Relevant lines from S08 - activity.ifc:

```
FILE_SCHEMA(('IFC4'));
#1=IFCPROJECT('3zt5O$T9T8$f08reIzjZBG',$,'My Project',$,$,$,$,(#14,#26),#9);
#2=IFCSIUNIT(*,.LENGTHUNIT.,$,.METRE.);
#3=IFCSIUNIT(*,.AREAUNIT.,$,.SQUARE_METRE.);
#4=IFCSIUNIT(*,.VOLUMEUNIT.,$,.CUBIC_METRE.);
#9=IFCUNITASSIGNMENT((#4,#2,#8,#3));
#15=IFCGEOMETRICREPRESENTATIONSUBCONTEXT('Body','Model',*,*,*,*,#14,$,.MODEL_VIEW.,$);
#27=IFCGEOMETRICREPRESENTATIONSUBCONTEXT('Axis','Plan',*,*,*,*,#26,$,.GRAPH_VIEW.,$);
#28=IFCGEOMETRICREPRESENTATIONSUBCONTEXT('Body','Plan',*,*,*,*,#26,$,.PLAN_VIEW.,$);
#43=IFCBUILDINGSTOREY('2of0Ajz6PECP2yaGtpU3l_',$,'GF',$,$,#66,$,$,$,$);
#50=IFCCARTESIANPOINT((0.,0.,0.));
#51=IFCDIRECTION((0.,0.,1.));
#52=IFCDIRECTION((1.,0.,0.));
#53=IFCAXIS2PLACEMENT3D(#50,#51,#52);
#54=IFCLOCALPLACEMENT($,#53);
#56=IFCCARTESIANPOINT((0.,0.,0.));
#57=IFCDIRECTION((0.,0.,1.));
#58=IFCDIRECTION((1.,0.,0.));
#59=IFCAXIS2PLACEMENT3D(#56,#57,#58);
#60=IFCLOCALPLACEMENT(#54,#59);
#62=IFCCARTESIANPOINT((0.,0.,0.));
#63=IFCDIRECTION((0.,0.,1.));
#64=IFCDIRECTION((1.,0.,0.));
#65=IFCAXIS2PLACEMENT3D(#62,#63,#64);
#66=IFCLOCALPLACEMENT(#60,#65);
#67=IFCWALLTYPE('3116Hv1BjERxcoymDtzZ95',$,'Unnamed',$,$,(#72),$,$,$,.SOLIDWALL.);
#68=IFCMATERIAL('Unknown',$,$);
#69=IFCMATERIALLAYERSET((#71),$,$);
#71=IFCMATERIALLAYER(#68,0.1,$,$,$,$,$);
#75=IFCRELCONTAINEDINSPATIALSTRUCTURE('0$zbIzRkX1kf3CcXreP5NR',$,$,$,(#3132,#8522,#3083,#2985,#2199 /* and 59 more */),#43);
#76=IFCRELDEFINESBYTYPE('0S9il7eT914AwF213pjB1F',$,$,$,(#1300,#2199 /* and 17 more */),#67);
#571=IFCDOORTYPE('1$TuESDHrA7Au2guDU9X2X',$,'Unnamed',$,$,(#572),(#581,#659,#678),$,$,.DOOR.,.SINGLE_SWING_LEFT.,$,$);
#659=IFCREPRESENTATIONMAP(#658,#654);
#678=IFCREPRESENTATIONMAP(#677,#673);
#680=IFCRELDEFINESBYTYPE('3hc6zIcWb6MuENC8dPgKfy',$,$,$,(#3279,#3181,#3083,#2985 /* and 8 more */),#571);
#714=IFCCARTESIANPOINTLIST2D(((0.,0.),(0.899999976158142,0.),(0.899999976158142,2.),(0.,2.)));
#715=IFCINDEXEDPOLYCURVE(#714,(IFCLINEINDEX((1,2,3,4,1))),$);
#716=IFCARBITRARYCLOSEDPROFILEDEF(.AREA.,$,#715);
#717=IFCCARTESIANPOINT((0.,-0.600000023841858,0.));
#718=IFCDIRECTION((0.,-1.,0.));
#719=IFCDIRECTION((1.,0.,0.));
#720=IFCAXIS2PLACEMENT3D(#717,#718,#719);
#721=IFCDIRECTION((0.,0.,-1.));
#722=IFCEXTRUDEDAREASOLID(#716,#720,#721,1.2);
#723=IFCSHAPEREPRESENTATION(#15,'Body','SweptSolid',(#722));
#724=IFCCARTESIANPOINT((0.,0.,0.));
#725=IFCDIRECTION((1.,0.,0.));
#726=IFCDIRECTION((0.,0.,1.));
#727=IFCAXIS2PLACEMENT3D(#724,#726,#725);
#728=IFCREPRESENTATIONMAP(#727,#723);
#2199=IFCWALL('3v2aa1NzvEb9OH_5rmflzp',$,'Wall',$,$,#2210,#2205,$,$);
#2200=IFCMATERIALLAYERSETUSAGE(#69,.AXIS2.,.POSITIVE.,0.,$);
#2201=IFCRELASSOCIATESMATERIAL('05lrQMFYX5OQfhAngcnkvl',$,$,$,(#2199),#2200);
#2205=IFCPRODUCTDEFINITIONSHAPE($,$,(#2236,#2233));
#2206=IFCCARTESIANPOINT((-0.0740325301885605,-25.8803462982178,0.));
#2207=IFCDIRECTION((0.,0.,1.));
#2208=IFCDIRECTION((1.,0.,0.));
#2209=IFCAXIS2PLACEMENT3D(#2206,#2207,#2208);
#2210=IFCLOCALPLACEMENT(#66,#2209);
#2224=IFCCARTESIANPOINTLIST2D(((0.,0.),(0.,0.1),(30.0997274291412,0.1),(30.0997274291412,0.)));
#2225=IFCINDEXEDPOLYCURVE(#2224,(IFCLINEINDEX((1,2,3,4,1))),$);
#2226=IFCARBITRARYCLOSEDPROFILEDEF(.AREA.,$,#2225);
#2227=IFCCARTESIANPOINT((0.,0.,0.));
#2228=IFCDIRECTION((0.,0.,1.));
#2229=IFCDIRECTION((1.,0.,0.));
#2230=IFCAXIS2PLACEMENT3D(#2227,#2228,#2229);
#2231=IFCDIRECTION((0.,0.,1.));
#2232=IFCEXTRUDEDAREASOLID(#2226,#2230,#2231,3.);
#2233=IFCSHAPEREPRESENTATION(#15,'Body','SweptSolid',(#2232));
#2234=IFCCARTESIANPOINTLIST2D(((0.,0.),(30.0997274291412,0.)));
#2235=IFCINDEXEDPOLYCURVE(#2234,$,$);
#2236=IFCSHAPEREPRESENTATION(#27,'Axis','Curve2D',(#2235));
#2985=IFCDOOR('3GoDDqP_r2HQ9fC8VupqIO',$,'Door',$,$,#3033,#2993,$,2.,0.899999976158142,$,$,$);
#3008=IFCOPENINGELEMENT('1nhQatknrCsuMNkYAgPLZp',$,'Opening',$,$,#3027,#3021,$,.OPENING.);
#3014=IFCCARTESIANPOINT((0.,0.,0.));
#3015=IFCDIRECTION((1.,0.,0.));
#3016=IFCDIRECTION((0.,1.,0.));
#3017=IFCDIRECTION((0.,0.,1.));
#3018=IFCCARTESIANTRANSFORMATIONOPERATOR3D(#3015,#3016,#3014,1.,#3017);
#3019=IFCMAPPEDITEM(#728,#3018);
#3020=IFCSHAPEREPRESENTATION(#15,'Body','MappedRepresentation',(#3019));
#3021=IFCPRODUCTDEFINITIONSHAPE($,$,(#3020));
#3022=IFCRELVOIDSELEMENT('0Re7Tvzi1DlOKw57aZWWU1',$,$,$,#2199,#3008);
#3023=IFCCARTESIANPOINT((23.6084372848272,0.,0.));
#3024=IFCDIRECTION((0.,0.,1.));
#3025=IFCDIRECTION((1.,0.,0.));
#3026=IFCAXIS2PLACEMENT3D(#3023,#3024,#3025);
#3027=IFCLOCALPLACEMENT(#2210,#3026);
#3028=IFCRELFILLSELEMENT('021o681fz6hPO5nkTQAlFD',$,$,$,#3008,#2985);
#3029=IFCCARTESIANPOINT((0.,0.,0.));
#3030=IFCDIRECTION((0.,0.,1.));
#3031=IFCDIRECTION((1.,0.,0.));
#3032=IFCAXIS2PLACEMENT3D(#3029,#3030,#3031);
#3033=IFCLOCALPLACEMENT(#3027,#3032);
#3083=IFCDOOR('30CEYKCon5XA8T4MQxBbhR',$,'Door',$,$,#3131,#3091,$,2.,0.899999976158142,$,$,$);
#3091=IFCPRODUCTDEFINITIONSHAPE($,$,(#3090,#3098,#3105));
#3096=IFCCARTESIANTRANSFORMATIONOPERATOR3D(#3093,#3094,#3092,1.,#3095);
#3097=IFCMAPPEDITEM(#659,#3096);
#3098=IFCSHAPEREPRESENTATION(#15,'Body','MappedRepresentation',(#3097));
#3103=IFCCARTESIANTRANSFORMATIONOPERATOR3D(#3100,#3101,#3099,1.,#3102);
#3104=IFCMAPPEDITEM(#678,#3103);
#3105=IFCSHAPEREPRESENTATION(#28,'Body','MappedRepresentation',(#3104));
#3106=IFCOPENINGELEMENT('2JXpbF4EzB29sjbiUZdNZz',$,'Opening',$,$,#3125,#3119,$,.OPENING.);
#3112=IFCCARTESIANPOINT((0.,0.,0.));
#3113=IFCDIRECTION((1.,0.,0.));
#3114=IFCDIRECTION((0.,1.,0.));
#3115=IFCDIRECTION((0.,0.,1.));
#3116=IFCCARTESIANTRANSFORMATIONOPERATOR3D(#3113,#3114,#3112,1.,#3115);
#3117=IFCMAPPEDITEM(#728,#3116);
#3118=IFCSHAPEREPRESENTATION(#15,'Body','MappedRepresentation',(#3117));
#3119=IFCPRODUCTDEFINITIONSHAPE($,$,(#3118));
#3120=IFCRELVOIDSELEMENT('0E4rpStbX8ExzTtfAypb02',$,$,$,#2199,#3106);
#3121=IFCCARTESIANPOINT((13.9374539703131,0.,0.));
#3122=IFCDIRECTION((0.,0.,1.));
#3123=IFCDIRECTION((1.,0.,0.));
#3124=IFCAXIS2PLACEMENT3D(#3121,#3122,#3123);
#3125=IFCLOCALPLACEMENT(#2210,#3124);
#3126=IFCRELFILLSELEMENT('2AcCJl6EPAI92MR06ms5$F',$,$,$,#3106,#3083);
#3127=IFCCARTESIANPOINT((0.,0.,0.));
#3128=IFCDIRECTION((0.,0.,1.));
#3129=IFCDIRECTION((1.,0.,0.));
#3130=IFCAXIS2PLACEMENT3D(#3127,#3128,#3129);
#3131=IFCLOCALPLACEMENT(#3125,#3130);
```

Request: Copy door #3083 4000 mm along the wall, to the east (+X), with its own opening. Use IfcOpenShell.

```python
import ifcopenshell
import ifcopenshell.api.feature
import ifcopenshell.api.geometry
import ifcopenshell.api.root
import ifcopenshell.geom
import ifcopenshell.util.element
import ifcopenshell.util.placement
import ifcopenshell.util.shape
import ifcopenshell.util.unit

model = ifcopenshell.open("S08 - activity.ifc")
unit_scale = ifcopenshell.util.unit.calculate_unit_scale(model)
settings = ifcopenshell.geom.settings()


def volume(element):
    """Net volume in cubic metres, openings subtracted."""
    shape = ifcopenshell.geom.create_shape(settings, element)
    return ifcopenshell.util.shape.get_volume(shape.geometry)


door = model.by_guid("30CEYKCon5XA8T4MQxBbhR")
opening = door.FillsVoids[0].RelatingOpeningElement
wall = opening.VoidsElements[0].RelatingBuildingElement
before = volume(wall)
shift = ifcopenshell.util.placement.get_local_placement(wall.ObjectPlacement)[:3, 0] * 4 / unit_scale

# copy_class copies the void relationship, type, container and properties, but no geometry.
new_opening = ifcopenshell.api.root.copy_class(model, product=opening)
new_opening.Representation = ifcopenshell.util.element.copy_deep(
    model, opening.Representation, exclude=["IfcGeometricRepresentationContext", "IfcRepresentationMap"]
)
new_door = ifcopenshell.api.root.copy_class(model, product=door)
new_door.Representation = ifcopenshell.util.element.copy_deep(
    model, door.Representation, exclude=["IfcGeometricRepresentationContext", "IfcRepresentationMap"]
)
ifcopenshell.api.feature.add_filling(model, opening=new_opening, element=new_door)

for old, new in ((opening, new_opening), (door, new_door)):
    matrix = ifcopenshell.util.placement.get_local_placement(old.ObjectPlacement)
    matrix[:3, 3] += shift
    ifcopenshell.api.geometry.edit_object_placement(model, product=new, matrix=matrix, is_si=False)

after = volume(wall)

print(f"wall volume {before:.3f} -> {after:.3f} m3")

model.write("S08 - activity_edited.ifc")
```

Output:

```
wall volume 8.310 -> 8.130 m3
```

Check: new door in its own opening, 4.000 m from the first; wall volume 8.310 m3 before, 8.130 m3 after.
